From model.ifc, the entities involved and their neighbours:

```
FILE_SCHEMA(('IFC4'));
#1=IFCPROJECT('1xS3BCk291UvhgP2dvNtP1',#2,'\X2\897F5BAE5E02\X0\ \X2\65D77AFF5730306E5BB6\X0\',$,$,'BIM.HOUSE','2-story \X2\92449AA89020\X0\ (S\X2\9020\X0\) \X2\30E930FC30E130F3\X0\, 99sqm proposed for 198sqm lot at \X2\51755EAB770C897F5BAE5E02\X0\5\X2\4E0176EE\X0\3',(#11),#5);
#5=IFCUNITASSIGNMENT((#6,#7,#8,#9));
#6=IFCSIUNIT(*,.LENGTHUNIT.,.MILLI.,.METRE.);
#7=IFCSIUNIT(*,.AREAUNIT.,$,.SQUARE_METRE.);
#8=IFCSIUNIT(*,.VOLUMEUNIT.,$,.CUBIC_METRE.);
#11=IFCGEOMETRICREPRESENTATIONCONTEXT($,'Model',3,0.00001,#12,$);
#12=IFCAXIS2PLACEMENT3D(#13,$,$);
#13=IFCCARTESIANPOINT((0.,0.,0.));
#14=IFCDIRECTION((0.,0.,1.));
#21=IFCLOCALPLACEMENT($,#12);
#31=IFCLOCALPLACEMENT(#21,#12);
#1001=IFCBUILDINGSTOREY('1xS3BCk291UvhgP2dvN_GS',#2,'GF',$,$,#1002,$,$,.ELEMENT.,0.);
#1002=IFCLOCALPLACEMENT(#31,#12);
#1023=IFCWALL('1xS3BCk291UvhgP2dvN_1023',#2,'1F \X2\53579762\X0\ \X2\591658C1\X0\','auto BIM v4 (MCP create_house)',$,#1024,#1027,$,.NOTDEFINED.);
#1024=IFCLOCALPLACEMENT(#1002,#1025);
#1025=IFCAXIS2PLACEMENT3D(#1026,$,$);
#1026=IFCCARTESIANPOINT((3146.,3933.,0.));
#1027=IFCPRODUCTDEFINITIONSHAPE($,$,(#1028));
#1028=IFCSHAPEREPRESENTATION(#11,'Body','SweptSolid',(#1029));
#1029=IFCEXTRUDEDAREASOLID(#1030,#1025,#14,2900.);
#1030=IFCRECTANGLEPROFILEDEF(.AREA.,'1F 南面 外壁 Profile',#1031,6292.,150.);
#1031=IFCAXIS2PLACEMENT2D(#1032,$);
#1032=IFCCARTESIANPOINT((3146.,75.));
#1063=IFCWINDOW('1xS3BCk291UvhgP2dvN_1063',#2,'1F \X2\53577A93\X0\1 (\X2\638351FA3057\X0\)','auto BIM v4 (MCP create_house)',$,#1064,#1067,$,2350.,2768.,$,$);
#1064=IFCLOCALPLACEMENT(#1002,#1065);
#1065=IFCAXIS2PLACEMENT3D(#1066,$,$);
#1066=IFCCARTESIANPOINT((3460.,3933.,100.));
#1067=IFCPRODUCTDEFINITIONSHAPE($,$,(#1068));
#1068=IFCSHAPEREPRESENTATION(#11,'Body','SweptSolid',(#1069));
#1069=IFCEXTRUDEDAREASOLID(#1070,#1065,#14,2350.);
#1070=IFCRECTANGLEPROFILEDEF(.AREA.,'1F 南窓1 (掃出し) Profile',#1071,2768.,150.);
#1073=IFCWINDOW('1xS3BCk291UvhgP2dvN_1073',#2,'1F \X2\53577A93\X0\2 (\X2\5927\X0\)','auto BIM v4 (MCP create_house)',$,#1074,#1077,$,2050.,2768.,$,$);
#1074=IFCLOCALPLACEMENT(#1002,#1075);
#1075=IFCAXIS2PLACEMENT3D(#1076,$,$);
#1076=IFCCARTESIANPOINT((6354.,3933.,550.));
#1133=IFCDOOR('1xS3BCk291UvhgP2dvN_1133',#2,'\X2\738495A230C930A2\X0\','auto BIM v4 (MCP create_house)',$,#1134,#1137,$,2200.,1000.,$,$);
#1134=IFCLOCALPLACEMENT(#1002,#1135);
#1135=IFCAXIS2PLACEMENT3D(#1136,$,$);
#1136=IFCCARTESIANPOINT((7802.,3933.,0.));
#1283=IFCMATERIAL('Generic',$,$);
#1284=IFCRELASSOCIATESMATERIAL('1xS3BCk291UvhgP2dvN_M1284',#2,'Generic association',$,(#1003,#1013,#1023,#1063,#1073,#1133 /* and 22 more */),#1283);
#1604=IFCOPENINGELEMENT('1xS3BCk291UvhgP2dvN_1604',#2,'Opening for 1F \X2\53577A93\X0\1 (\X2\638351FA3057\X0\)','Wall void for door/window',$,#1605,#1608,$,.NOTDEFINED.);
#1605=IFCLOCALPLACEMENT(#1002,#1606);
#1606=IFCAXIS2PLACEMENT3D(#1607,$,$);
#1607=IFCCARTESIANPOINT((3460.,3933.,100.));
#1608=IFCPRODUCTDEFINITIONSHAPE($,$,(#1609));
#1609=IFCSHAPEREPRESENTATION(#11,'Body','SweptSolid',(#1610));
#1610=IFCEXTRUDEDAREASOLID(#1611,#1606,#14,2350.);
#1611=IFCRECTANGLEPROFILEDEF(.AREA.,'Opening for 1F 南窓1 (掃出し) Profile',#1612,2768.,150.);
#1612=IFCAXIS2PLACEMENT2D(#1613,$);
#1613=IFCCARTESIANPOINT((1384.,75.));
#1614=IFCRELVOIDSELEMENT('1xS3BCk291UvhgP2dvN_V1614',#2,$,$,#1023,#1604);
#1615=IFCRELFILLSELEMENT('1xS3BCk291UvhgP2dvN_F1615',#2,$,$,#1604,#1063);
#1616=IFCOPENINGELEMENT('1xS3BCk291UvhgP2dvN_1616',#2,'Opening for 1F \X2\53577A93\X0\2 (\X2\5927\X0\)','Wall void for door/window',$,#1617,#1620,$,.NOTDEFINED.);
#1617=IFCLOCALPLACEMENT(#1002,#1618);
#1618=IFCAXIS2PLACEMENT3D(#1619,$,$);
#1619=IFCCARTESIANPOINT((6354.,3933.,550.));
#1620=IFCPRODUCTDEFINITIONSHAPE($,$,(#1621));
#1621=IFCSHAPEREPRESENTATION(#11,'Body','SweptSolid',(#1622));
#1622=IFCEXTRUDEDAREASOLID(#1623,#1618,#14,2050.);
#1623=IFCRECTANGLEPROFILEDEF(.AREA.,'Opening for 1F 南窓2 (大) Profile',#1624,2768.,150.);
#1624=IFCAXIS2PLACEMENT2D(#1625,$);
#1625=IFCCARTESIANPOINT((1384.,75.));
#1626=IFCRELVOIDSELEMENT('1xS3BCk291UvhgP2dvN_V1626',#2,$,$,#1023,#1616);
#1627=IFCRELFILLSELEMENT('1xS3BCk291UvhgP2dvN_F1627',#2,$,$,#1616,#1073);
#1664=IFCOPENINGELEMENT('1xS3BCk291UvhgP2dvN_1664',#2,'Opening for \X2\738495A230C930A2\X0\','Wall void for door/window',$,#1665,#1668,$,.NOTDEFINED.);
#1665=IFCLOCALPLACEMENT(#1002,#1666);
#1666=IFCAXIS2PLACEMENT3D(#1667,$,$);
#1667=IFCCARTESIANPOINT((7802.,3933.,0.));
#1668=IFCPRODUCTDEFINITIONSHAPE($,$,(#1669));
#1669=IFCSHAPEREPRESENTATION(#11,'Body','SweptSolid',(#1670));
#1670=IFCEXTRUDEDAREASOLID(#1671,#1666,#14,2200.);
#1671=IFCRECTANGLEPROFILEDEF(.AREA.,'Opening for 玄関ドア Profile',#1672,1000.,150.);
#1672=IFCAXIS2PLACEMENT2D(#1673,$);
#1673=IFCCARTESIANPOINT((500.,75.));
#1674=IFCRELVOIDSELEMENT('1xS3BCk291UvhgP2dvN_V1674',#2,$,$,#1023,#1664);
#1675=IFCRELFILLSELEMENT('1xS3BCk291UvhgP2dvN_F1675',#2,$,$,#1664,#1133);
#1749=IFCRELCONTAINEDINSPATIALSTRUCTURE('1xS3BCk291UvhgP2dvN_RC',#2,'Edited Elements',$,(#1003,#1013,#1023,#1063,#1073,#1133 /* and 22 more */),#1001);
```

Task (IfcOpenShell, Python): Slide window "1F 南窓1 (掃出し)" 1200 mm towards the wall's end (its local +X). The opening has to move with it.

```python
import ifcopenshell
import ifcopenshell.api.geometry
import ifcopenshell.util.placement
import ifcopenshell.util.unit

model = ifcopenshell.open("model.ifc")
unit_scale = ifcopenshell.util.unit.calculate_unit_scale(model)

window = model.by_id(1063)
opening = window.FillsVoids[0].RelatingOpeningElement
wall = opening.VoidsElements[0].RelatingBuildingElement

wall_matrix = ifcopenshell.util.placement.get_local_placement(wall.ObjectPlacement)
shift = wall_matrix[:3, 0] * 1.2 / unit_scale
before = ifcopenshell.util.placement.get_local_placement(window.ObjectPlacement)[:3, 3].copy()

# The window is not placed relative to its opening, so move both.
for product in (opening, window):
    matrix = ifcopenshell.util.placement.get_local_placement(product.ObjectPlacement)
    matrix[:3, 3] += shift
    ifcopenshell.api.geometry.edit_object_placement(model, product=product, matrix=matrix, is_si=False)

after = ifcopenshell.util.placement.get_local_placement(window.ObjectPlacement)[:3, 3]
print("window moved by", (after - before).round(3) + 0.0)

model.write("model_updated.ifc")
```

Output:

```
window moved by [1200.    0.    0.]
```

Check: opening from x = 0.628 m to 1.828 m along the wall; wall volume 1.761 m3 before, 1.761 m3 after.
